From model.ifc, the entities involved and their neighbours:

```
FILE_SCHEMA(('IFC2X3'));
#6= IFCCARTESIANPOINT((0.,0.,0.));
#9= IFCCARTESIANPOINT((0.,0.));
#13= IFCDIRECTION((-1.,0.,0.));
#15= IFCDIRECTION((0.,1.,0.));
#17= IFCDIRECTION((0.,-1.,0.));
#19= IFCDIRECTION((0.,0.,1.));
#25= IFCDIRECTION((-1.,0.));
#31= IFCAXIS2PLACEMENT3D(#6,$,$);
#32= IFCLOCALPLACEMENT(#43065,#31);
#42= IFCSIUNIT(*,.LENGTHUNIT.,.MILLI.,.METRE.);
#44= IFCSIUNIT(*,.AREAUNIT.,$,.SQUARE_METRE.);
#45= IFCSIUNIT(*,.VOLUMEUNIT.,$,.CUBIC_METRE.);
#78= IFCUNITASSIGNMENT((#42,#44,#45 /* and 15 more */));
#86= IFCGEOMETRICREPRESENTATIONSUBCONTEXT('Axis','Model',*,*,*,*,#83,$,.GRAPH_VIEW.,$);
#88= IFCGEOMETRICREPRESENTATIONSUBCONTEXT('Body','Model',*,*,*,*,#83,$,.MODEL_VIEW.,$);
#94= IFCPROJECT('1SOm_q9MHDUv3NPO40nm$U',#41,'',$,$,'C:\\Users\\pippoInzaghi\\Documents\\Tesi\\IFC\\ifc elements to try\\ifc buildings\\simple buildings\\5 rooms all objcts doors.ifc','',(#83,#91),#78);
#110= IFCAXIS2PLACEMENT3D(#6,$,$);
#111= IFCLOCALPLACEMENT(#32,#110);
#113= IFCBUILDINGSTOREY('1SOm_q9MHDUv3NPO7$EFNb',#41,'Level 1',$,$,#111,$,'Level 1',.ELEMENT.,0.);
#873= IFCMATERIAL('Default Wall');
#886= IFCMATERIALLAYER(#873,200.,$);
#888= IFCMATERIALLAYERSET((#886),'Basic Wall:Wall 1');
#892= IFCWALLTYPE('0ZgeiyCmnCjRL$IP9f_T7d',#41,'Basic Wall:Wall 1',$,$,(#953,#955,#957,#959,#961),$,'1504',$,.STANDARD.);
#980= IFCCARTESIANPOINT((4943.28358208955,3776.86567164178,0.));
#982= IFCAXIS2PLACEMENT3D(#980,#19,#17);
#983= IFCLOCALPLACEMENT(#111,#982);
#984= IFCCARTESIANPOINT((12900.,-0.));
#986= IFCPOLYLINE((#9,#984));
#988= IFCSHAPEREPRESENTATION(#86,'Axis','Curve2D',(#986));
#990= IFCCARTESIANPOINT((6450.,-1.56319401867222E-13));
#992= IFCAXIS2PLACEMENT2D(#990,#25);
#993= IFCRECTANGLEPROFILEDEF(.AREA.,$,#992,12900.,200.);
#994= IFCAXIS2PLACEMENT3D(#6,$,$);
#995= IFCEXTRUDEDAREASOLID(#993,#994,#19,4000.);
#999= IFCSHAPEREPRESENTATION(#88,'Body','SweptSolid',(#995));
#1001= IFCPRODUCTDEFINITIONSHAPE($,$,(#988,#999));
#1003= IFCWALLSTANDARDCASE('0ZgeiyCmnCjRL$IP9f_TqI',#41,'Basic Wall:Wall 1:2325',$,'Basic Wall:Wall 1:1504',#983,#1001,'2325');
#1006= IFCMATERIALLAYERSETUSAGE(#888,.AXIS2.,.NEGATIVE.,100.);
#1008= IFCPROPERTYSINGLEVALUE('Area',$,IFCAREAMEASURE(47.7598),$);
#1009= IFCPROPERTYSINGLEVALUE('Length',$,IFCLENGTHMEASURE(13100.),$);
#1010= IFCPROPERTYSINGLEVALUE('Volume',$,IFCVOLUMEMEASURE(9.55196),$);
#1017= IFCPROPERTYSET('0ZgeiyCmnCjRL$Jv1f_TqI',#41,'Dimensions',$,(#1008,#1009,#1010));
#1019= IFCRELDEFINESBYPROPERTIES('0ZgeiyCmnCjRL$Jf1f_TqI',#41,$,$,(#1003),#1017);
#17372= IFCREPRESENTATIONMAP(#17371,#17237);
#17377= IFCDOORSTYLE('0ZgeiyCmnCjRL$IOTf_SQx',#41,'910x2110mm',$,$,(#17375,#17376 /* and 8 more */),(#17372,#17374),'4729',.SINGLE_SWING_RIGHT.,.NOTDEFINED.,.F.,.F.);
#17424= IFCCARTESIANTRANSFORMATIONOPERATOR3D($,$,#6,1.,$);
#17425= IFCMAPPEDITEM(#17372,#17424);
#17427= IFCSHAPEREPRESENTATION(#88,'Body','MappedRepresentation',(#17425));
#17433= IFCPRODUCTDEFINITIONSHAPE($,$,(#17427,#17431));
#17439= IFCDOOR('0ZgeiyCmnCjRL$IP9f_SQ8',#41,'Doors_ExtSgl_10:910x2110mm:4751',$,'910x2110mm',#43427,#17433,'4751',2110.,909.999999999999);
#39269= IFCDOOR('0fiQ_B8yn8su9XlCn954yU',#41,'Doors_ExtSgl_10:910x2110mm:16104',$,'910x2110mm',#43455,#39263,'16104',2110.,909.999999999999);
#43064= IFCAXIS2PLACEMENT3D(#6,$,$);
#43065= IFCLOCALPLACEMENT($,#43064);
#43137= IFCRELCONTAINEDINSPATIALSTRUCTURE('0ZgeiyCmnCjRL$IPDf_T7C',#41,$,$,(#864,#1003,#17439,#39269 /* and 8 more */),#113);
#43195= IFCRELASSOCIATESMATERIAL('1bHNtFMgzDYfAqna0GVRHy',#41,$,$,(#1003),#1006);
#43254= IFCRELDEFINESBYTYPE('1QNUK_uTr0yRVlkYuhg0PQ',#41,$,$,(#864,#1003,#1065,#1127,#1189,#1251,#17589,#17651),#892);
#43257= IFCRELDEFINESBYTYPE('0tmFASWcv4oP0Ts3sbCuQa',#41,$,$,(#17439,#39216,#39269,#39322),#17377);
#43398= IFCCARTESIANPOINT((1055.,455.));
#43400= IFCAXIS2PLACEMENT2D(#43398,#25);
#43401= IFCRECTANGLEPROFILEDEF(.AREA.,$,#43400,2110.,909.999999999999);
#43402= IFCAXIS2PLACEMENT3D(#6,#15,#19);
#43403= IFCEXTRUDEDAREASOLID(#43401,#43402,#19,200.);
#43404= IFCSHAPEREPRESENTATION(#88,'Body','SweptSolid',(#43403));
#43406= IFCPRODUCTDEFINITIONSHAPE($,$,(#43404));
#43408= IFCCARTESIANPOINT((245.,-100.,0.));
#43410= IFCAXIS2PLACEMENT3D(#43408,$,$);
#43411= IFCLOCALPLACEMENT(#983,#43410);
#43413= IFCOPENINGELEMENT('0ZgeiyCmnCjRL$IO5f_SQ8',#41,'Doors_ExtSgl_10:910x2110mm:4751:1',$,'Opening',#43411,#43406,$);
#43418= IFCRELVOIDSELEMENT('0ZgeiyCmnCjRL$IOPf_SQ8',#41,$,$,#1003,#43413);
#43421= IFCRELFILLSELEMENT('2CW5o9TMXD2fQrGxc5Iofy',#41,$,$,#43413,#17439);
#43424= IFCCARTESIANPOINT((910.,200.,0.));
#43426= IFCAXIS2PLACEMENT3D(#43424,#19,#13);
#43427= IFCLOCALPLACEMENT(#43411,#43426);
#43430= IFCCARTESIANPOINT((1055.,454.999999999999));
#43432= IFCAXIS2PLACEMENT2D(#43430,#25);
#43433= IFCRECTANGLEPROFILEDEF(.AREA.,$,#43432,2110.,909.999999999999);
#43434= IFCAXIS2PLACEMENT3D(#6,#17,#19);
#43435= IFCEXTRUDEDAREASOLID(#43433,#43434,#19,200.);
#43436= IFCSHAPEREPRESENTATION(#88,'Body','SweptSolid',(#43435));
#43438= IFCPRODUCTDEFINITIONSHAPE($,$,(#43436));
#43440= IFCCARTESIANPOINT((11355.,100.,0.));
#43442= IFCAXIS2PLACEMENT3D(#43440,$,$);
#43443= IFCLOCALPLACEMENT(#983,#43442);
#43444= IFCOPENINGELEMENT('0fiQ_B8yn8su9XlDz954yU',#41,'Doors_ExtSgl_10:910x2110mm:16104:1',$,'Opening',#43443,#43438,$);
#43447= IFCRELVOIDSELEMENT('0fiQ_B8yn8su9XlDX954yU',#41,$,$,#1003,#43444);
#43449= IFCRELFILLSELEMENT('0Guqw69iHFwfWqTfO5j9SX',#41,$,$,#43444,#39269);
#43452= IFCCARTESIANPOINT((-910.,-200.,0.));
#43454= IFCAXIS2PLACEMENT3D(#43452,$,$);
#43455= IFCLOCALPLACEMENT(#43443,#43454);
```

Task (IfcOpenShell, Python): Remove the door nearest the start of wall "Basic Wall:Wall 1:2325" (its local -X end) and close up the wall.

```python
import ifcopenshell
import ifcopenshell.api.feature
import ifcopenshell.api.pset
import ifcopenshell.api.root
import ifcopenshell.geom
import ifcopenshell.util.element
import ifcopenshell.util.shape
import ifcopenshell.util.unit

model = ifcopenshell.open("model.ifc")
area_scale = ifcopenshell.util.unit.calculate_unit_scale(model, "AREAUNIT")
volume_scale = ifcopenshell.util.unit.calculate_unit_scale(model, "VOLUMEUNIT")
settings = ifcopenshell.geom.settings()


def volume(element):
    """Net volume in cubic metres, openings subtracted."""
    shape = ifcopenshell.geom.create_shape(settings, element)
    return ifcopenshell.util.shape.get_volume(shape.geometry)


door = model.by_guid("0ZgeiyCmnCjRL$IP9f_SQ8")
opening = door.FillsVoids[0].RelatingOpeningElement
wall = opening.VoidsElements[0].RelatingBuildingElement
before = volume(wall)

ifcopenshell.api.root.remove_product(model, product=door)
ifcopenshell.api.feature.remove_feature(model, feature=opening)

after = volume(wall)
thickness = 0.2  # wall thickness in metres

# Update the wall's stored quantities.
pset = model.by_id(ifcopenshell.util.element.get_pset(wall, "Dimensions", should_inherit=False)["id"])
ifcopenshell.api.pset.edit_pset(model, pset=pset, properties={
    "Area": model.create_entity("IfcAreaMeasure", after / thickness / area_scale),
    "Volume": model.create_entity("IfcVolumeMeasure", after / volume_scale),
})

print(f"wall volume {before:.3f} -> {after:.3f} m3")

model.write("model_v2.ifc")
```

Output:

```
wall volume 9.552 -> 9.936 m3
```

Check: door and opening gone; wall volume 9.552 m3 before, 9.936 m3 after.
